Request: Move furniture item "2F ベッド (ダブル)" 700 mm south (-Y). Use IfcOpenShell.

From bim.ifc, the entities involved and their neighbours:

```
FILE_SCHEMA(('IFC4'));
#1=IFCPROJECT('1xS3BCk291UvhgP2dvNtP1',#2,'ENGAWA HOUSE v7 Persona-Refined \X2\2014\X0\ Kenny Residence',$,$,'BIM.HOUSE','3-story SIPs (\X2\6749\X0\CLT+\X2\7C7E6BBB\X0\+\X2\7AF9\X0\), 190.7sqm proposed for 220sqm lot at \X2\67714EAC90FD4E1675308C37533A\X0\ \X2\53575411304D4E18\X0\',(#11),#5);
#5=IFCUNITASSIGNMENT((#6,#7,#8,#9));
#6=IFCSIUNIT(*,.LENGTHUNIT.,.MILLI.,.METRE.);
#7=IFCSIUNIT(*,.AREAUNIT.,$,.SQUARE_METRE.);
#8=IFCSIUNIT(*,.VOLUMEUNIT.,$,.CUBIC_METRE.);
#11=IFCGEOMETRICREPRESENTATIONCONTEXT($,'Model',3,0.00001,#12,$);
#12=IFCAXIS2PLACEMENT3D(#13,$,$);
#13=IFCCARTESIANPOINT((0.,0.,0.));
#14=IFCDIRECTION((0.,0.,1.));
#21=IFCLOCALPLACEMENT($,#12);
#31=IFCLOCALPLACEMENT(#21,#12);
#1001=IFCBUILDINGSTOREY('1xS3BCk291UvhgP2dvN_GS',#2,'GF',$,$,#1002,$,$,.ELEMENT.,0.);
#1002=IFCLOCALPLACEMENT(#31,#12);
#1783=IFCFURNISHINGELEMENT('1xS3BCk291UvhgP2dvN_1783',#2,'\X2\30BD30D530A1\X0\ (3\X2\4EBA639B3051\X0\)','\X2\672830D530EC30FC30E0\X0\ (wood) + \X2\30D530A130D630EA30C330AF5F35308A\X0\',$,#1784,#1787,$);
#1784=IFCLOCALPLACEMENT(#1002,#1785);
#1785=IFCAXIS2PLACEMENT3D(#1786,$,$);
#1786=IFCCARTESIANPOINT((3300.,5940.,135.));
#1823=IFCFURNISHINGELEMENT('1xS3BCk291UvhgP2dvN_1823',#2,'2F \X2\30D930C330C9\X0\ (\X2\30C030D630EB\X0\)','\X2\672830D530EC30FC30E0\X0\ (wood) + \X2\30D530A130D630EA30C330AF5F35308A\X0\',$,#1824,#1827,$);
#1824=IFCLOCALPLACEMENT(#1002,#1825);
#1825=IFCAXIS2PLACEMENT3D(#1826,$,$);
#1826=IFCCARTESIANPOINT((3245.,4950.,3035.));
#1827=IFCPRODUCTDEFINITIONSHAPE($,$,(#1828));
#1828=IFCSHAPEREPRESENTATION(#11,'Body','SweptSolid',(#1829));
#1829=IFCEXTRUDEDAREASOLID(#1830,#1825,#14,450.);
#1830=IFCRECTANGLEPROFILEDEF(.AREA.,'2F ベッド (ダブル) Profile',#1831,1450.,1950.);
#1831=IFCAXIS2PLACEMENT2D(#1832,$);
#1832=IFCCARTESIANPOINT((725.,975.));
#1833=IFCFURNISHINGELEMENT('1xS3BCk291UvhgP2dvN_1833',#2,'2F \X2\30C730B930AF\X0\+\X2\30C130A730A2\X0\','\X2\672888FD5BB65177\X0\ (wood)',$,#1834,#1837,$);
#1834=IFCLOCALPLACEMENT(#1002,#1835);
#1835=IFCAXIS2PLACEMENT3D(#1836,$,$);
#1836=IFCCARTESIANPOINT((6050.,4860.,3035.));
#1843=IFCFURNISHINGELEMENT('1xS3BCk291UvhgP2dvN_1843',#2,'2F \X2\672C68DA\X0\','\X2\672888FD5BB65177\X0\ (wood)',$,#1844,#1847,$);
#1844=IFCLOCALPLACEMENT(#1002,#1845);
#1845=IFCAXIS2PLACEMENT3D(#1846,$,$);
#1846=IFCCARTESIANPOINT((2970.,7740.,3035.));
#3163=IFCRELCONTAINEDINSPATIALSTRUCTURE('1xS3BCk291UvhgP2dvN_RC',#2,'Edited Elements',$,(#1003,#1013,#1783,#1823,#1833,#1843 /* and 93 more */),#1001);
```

```python
import ifcopenshell
import ifcopenshell.api.geometry
import ifcopenshell.util.placement

model = ifcopenshell.open("bim.ifc")

item = model.by_guid("1xS3BCk291UvhgP2dvN_1823")
matrix = ifcopenshell.util.placement.get_local_placement(item.ObjectPlacement)
matrix[1, 3] -= 700.0
ifcopenshell.api.geometry.edit_object_placement(model, product=item, matrix=matrix, is_si=False)

print(ifcopenshell.util.placement.get_local_placement(item.ObjectPlacement).round(3) + 0.0)

model.write("bim_rev.ifc")
```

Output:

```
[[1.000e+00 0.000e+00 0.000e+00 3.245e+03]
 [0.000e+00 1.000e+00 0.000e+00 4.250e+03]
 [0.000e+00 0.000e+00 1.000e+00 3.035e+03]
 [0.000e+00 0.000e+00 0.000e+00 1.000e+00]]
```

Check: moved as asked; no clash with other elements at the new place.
